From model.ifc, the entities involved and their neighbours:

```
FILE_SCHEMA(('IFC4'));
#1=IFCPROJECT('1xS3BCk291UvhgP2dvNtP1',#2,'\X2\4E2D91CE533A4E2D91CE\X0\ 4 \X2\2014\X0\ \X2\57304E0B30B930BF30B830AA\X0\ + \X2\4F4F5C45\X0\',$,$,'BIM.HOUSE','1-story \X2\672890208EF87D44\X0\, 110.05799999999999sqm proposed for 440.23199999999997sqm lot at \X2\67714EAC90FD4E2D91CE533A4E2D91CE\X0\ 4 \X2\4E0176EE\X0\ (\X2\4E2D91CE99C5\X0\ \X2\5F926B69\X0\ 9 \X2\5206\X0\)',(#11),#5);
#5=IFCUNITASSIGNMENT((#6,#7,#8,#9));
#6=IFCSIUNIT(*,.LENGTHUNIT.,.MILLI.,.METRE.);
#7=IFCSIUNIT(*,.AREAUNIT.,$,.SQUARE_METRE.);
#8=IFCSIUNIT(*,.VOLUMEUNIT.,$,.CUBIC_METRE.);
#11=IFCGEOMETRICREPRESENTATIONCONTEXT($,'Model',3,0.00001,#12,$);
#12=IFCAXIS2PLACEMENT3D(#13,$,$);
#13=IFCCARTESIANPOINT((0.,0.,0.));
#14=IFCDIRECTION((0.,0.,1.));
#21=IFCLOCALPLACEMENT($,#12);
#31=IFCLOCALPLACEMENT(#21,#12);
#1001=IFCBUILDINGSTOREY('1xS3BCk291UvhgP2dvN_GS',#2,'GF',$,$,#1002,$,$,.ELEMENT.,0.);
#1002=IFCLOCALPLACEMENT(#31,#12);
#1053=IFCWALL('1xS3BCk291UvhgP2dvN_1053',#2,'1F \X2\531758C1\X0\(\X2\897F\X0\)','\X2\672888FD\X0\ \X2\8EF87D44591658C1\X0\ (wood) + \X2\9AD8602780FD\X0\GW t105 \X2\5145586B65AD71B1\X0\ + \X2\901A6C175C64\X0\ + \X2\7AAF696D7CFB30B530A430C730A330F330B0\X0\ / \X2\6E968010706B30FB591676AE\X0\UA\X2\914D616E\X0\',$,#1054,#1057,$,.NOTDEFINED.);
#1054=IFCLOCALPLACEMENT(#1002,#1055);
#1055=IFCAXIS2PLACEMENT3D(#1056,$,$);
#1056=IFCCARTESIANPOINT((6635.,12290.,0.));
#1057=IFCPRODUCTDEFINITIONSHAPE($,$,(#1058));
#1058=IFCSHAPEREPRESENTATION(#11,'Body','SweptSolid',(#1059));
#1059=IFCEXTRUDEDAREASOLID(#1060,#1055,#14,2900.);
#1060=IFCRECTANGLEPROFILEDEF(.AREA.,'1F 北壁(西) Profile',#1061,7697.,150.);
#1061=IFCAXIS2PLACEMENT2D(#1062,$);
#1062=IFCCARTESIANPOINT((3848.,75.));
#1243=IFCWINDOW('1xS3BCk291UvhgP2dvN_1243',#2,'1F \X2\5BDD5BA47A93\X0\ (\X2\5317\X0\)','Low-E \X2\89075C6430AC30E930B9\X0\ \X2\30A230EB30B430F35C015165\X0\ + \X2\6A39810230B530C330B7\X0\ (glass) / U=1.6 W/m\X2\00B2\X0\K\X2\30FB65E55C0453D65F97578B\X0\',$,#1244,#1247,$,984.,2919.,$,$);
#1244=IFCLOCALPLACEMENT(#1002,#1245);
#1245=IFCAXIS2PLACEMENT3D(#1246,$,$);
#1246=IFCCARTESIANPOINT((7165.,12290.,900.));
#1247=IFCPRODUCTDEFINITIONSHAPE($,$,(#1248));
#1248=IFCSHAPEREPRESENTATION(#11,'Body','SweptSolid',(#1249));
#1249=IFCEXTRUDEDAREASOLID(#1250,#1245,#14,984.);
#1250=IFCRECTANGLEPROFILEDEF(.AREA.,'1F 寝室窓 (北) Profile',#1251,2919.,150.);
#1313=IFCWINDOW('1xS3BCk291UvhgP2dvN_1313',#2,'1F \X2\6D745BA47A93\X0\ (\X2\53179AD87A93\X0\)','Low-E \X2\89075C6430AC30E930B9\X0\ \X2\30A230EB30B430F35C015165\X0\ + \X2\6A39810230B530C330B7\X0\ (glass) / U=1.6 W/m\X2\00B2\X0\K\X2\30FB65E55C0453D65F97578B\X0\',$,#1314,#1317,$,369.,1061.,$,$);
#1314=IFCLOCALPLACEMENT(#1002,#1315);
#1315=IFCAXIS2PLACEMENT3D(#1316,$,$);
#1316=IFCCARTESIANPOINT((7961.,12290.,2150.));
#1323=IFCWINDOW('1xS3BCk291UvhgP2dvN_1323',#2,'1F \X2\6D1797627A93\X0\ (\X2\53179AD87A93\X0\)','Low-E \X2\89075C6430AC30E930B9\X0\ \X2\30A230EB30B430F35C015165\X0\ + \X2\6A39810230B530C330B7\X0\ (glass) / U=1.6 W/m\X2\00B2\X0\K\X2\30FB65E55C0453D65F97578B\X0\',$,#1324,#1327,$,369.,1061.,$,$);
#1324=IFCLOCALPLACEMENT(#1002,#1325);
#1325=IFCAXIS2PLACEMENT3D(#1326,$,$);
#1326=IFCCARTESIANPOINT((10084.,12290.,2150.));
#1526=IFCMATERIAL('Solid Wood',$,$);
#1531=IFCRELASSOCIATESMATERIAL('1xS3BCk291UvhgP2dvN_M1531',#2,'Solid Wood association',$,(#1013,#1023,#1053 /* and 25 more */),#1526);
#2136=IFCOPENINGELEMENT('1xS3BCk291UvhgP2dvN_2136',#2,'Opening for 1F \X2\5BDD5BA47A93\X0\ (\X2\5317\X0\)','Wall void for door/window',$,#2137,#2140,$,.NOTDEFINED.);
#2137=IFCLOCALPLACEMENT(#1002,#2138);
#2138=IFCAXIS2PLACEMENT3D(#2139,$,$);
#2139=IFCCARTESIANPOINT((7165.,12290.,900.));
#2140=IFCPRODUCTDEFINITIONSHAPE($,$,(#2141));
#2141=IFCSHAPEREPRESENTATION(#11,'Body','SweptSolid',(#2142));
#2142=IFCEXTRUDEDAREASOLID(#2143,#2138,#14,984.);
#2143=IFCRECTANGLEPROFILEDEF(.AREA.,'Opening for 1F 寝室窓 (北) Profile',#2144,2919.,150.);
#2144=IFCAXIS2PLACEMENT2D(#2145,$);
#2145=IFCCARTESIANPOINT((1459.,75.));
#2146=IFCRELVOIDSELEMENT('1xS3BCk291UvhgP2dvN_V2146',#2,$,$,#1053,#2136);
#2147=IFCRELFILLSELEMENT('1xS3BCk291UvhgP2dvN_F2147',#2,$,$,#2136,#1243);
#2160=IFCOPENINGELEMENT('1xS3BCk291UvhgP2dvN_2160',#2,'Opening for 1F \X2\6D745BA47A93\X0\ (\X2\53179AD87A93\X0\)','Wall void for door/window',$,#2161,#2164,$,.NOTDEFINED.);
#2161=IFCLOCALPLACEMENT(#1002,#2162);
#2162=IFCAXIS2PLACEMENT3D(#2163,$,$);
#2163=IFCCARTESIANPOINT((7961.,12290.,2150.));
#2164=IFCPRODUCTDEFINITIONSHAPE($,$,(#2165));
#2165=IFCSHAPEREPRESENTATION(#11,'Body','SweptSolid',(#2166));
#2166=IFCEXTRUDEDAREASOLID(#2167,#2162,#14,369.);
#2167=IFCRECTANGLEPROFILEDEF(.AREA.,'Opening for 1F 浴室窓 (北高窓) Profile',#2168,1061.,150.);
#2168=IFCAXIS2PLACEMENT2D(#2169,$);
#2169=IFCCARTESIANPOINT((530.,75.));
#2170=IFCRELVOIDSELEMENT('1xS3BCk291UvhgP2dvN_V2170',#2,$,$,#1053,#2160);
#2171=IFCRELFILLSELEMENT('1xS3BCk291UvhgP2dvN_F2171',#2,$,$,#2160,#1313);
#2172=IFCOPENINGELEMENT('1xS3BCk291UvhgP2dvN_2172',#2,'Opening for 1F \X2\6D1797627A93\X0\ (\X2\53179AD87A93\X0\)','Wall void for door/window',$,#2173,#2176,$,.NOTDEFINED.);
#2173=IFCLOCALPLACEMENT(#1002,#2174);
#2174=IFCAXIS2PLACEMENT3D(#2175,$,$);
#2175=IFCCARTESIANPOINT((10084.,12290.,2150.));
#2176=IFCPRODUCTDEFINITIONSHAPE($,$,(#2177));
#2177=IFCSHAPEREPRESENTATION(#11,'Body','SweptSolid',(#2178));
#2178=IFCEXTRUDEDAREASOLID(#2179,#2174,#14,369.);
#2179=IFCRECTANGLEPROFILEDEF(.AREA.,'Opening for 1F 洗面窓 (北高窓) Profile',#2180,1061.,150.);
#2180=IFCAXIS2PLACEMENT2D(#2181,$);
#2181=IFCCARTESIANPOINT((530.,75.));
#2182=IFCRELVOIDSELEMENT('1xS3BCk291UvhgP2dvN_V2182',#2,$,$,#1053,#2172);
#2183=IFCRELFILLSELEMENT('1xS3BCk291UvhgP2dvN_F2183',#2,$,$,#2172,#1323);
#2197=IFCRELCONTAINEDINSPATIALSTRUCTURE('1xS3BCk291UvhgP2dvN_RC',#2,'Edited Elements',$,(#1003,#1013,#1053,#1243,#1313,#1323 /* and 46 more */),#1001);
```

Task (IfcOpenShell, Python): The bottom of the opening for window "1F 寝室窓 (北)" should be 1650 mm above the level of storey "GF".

```python
import numpy as np
import ifcopenshell
import ifcopenshell.api.geometry
import ifcopenshell.geom
import ifcopenshell.util.element
import ifcopenshell.util.placement
import ifcopenshell.util.shape
import ifcopenshell.util.unit

model = ifcopenshell.open("model.ifc")
unit_scale = ifcopenshell.util.unit.calculate_unit_scale(model)

window = model.by_guid("1xS3BCk291UvhgP2dvN_1243")
opening = window.FillsVoids[0].RelatingOpeningElement
storey = ifcopenshell.util.element.get_container(window, ifc_class="IfcBuildingStorey")
level = ifcopenshell.util.placement.get_local_placement(storey.ObjectPlacement)[2, 3]

# The opening's origin need not be at the sill, so measure its lowest point.
shape = ifcopenshell.geom.create_shape(ifcopenshell.geom.settings(), opening)
bottom = ifcopenshell.util.shape.get_shape_bottom_elevation(shape, shape.geometry) / unit_scale
dz = level + 1.65 / unit_scale - bottom

shift = np.array([0.0, 0.0, dz])
# The window is not placed relative to its opening, so move both.
for product in (opening, window):
    matrix = ifcopenshell.util.placement.get_local_placement(product.ObjectPlacement)
    matrix[:3, 3] += shift
    ifcopenshell.api.geometry.edit_object_placement(model, product=product, matrix=matrix, is_si=False)

print(f"moved by {dz * unit_scale:+.3f} m")

model.write("model_v2.ifc")
```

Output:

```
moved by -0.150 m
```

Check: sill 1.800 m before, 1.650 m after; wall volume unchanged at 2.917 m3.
